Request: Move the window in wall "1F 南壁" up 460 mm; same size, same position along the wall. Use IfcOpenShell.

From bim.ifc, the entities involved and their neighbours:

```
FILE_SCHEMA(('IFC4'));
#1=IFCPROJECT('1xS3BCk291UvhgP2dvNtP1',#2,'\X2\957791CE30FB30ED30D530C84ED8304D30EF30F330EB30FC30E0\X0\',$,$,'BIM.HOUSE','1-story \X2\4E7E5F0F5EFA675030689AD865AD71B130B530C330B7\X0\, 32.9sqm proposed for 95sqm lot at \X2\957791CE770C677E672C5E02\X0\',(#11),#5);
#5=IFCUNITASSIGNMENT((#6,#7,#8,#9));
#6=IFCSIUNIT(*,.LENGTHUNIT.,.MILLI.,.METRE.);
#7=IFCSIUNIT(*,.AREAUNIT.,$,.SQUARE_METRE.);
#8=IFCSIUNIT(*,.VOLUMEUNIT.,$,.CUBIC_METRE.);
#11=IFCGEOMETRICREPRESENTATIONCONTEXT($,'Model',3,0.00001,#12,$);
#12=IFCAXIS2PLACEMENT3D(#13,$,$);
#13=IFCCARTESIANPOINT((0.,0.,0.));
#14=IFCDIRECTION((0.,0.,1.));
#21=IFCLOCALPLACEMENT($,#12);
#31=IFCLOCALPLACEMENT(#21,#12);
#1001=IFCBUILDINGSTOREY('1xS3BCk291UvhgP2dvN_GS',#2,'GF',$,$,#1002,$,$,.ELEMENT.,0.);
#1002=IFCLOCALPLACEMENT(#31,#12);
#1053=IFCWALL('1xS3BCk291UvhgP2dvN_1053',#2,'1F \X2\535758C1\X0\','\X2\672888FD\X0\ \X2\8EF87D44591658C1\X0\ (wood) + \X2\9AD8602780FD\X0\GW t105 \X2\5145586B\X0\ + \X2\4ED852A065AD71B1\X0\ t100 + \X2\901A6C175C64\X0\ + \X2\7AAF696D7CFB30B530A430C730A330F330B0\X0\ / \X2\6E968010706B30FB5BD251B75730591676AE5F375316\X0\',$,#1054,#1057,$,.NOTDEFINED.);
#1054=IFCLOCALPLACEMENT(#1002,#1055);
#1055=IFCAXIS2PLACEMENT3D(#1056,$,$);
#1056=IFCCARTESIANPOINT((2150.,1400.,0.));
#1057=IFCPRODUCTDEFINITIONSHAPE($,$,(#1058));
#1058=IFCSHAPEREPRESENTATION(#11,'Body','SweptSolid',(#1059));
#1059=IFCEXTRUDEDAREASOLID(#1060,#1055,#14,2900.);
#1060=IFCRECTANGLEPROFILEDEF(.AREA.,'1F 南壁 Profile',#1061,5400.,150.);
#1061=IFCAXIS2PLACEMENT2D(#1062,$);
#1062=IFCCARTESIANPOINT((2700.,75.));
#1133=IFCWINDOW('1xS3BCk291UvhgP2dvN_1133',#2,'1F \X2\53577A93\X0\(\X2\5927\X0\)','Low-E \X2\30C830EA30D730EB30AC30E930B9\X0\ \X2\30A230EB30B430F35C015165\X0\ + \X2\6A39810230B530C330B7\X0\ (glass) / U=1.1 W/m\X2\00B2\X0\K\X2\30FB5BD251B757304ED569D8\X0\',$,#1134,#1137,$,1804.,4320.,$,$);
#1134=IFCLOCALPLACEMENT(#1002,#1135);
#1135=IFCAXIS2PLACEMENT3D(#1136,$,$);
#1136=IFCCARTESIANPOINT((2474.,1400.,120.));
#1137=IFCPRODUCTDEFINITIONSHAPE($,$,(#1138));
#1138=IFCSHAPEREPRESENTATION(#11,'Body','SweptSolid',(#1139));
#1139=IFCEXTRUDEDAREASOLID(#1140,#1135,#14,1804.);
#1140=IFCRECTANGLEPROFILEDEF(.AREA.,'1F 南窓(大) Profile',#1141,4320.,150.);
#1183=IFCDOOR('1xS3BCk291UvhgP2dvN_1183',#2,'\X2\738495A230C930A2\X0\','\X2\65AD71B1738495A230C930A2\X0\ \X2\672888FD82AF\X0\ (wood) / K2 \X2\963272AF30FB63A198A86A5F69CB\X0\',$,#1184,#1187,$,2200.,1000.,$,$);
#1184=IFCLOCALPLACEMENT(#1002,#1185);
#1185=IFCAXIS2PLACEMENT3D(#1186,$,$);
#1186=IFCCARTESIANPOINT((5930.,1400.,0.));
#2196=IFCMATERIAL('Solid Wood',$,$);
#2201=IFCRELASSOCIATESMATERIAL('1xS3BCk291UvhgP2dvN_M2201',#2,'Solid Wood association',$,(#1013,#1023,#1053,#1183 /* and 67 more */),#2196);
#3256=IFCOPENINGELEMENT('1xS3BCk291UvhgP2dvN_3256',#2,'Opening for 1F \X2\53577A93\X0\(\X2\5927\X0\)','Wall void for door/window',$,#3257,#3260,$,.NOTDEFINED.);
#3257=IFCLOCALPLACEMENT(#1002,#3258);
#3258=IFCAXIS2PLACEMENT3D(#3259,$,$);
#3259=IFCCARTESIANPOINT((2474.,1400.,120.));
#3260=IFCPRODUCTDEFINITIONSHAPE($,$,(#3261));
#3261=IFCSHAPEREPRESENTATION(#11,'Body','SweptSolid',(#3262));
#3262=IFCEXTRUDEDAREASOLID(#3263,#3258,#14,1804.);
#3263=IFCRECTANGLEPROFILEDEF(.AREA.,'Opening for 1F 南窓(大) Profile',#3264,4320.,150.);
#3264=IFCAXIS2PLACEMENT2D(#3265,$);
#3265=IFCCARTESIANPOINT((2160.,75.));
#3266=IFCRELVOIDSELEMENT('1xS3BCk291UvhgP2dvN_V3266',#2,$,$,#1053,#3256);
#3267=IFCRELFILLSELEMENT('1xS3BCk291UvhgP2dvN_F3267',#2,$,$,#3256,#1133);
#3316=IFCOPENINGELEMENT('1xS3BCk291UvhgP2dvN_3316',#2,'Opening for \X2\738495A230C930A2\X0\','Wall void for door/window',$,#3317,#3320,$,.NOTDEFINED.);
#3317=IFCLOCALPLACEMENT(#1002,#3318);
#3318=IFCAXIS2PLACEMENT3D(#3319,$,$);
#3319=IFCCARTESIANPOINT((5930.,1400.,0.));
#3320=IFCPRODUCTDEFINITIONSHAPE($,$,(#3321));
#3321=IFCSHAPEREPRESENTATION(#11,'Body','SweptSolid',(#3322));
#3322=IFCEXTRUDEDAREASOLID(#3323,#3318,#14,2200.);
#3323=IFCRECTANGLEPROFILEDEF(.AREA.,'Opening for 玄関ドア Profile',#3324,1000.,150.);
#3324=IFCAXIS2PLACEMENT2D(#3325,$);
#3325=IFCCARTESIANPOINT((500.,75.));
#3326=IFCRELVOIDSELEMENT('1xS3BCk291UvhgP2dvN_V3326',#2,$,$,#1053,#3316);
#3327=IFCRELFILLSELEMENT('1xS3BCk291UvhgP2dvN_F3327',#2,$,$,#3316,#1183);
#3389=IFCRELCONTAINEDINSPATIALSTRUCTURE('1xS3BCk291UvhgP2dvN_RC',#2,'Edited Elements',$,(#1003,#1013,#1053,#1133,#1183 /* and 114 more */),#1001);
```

```python
import numpy as np
import ifcopenshell
import ifcopenshell.api.geometry
import ifcopenshell.util.placement
import ifcopenshell.util.unit

model = ifcopenshell.open("bim.ifc")
unit_scale = ifcopenshell.util.unit.calculate_unit_scale(model)

window = model.by_guid("1xS3BCk291UvhgP2dvN_1133")
opening = window.FillsVoids[0].RelatingOpeningElement
dz = 460.0

shift = np.array([0.0, 0.0, dz])
# The window is not placed relative to its opening, so move both.
for product in (opening, window):
    matrix = ifcopenshell.util.placement.get_local_placement(product.ObjectPlacement)
    matrix[:3, 3] += shift
    ifcopenshell.api.geometry.edit_object_placement(model, product=product, matrix=matrix, is_si=False)

print(f"moved by {dz * unit_scale:+.3f} m")

model.write("bim-out.ifc")
```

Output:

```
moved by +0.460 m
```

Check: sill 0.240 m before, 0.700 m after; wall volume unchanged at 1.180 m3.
